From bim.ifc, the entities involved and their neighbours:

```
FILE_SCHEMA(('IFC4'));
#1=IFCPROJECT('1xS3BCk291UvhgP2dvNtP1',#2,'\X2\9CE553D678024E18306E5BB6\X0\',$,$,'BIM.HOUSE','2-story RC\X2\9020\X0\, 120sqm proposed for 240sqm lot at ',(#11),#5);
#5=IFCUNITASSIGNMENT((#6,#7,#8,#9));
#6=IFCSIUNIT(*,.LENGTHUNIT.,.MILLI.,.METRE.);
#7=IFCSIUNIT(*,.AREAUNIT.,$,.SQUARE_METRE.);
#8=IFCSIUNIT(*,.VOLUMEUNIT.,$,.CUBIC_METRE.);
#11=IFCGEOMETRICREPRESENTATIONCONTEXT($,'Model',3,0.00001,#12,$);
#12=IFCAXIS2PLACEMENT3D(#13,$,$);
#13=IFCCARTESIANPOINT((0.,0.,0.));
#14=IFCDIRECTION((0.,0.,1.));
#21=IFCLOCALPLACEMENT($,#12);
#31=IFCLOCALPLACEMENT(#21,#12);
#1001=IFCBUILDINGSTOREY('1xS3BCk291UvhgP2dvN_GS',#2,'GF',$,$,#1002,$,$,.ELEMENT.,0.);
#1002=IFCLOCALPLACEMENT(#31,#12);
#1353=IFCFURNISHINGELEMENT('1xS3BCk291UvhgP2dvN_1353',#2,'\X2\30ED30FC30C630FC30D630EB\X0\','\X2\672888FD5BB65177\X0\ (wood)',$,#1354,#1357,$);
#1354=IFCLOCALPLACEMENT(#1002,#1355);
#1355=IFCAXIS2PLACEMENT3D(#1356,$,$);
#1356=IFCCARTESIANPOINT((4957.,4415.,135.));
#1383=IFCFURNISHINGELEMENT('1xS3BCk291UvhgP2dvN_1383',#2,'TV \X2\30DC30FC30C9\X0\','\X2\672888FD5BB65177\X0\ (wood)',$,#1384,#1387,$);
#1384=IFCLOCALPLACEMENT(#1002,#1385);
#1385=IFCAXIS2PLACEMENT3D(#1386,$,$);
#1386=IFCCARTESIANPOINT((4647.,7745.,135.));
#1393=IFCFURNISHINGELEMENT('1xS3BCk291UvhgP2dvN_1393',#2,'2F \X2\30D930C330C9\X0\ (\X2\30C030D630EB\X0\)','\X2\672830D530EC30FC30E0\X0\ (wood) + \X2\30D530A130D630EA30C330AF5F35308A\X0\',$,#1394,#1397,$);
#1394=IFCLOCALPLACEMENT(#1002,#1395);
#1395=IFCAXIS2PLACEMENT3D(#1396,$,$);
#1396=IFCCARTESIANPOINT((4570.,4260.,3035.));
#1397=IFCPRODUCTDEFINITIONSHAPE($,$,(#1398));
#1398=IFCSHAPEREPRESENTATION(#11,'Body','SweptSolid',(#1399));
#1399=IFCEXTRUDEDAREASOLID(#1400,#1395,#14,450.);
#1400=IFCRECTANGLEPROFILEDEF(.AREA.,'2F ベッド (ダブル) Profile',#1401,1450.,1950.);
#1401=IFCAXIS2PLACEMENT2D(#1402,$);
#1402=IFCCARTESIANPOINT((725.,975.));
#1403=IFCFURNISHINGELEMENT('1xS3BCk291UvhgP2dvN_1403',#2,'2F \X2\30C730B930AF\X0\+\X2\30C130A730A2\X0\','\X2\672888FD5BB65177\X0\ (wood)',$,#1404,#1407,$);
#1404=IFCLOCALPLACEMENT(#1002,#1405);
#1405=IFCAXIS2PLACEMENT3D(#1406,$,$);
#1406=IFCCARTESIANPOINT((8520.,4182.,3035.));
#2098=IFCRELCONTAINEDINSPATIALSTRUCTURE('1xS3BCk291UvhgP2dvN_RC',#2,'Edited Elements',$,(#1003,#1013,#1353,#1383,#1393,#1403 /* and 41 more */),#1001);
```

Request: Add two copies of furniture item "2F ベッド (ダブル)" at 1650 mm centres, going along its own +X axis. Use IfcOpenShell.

```python
import ifcopenshell
import ifcopenshell.api.geometry
import ifcopenshell.api.root
import ifcopenshell.util.element
import ifcopenshell.util.placement
import ifcopenshell.util.unit

model = ifcopenshell.open("bim.ifc")
unit_scale = ifcopenshell.util.unit.calculate_unit_scale(model)


def reuse_history(source, copy):
    """copy_class also copies each property set's owner history, people and application; keep the originals."""
    for rel in copy.IsDefinedBy:
        if rel.is_a("IfcRelDefinesByProperties") and (history := rel.RelatingPropertyDefinition.OwnerHistory):
            rel.RelatingPropertyDefinition.OwnerHistory = source.OwnerHistory
            ifcopenshell.util.element.remove_deep2(model, history)


source = model.by_guid("1xS3BCk291UvhgP2dvN_1393")
base = ifcopenshell.util.placement.get_local_placement(source.ObjectPlacement)
step = base[:3, 0] * 1.65 / unit_scale

for i in range(1, 3):
    copy = ifcopenshell.api.root.copy_class(model, product=source)
    copy.Representation = ifcopenshell.util.element.copy_deep(
        model, source.Representation, exclude=["IfcGeometricRepresentationContext", "IfcRepresentationMap"]
    )
    reuse_history(source, copy)
    matrix = base.copy()
    matrix[:3, 3] += i * step
    print("added at", matrix[:3, 3].round(3) + 0.0)
    ifcopenshell.api.geometry.edit_object_placement(model, product=copy, matrix=matrix, is_si=False)

model.write("bim_v2.ifc")
```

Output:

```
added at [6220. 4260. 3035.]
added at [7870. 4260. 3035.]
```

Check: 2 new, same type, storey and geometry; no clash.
